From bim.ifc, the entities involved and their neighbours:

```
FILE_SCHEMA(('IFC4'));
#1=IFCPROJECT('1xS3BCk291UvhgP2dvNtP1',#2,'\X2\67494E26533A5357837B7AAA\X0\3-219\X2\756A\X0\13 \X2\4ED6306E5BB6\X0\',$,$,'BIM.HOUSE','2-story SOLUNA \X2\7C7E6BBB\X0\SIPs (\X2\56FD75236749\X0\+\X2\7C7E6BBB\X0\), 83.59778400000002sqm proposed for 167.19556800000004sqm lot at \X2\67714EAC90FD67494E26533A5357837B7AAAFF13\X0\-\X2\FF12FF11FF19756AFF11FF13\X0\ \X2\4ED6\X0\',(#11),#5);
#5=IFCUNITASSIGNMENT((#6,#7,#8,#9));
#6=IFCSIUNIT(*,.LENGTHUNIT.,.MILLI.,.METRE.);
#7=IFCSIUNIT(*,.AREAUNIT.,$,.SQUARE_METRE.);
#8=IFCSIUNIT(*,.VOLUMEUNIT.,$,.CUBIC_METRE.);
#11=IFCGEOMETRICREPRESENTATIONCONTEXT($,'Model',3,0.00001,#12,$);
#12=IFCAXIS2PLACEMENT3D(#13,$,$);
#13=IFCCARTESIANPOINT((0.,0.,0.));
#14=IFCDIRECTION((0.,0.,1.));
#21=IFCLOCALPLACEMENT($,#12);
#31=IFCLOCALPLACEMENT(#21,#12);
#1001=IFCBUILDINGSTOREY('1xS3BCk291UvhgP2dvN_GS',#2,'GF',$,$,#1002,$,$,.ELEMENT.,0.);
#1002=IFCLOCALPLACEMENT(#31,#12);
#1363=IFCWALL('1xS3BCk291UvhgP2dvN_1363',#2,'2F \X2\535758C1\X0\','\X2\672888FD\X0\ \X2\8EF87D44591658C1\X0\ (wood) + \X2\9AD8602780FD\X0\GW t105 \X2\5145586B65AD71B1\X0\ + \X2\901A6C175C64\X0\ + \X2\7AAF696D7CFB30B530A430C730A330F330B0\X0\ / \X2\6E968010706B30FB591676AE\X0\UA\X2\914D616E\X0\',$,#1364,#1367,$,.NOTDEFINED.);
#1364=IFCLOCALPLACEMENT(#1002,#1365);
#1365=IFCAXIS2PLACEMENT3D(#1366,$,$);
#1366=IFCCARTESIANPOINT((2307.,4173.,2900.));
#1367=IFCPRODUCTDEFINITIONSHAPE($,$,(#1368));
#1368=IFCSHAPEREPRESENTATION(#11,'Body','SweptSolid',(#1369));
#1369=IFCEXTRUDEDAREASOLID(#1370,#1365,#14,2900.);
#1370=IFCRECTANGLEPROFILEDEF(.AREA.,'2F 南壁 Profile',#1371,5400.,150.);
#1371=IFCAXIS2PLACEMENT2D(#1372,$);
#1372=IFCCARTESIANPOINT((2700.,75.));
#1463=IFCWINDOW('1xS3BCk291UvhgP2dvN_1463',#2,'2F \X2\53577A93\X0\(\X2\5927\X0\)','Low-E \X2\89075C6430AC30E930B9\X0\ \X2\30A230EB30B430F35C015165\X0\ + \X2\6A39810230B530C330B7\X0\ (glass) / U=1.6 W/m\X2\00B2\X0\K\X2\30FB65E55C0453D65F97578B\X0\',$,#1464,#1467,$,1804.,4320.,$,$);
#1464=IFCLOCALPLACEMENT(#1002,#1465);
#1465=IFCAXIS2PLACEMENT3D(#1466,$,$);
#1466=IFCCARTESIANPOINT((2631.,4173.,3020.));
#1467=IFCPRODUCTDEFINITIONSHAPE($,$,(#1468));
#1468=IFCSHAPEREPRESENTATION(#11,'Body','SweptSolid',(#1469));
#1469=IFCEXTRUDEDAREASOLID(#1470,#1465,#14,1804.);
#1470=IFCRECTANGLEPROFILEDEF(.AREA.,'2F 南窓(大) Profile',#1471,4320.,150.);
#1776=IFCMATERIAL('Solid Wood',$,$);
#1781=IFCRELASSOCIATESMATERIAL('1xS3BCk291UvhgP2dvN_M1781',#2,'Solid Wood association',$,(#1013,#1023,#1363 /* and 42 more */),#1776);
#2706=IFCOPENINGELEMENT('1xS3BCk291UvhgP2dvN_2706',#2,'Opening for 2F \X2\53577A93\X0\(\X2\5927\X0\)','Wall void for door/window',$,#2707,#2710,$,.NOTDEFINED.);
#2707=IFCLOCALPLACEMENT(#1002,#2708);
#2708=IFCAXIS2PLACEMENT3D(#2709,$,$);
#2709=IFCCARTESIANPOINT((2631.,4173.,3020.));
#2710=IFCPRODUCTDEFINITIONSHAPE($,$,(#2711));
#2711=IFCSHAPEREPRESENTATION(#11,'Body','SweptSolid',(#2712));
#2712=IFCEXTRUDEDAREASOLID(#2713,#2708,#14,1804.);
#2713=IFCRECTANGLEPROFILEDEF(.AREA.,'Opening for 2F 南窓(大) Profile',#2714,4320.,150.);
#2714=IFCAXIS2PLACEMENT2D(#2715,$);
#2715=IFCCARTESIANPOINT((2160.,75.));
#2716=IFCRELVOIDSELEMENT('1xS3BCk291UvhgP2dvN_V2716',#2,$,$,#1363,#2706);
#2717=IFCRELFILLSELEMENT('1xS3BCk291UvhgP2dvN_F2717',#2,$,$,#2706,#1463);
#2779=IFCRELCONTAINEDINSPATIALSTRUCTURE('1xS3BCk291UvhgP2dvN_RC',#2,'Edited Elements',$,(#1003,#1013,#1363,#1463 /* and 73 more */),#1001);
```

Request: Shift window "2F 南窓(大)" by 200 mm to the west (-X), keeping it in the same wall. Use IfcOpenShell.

```python
import ifcopenshell
import ifcopenshell.api.geometry
import ifcopenshell.util.placement

model = ifcopenshell.open("bim.ifc")

window = model.by_id(1463)
opening = window.FillsVoids[0].RelatingOpeningElement
wall = opening.VoidsElements[0].RelatingBuildingElement

wall_matrix = ifcopenshell.util.placement.get_local_placement(wall.ObjectPlacement)
shift = wall_matrix[:3, 0] * -200.0
before = ifcopenshell.util.placement.get_local_placement(window.ObjectPlacement)[:3, 3].copy()

# The window is not placed relative to its opening, so move both.
for product in (opening, window):
    matrix = ifcopenshell.util.placement.get_local_placement(product.ObjectPlacement)
    matrix[:3, 3] += shift
    ifcopenshell.api.geometry.edit_object_placement(model, product=product, matrix=matrix, is_si=False)

after = ifcopenshell.util.placement.get_local_placement(window.ObjectPlacement)[:3, 3]
print("window moved by", (after - before).round(3) + 0.0)

model.write("bim-out.ifc")
```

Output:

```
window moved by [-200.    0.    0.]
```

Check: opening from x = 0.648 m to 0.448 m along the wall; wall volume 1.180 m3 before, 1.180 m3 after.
